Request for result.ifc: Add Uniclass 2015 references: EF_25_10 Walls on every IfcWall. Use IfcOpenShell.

First a look at what the model holds.

```python
import ifcopenshell

model = ifcopenshell.open("result.ifc")
print(model.schema)
print("classifications:", [c.Name for c in model.by_type("IfcClassification")])
for ifc_class in ("IfcDoor", "IfcRoof", "IfcStair", "IfcWall", "IfcWindow"):
    print(ifc_class, len(model.by_type(ifc_class)))
```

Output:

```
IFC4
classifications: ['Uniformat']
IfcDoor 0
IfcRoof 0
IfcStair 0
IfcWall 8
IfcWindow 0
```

```python
import ifcopenshell
import ifcopenshell.api.classification

model = ifcopenshell.open("result.ifc")

system = ifcopenshell.api.classification.add_classification(model, classification="Uniclass 2015")

codes = {
    "IfcWall": ("EF_25_10", "Walls"),
}
for ifc_class, (code, name) in codes.items():
    products = model.by_type(ifc_class)
    ifcopenshell.api.classification.add_reference(
        model, products=products, classification=system, identification=code, name=name
    )
    print(code, len(products))

model.write("result_rev.ifc")
```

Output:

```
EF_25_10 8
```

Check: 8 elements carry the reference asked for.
